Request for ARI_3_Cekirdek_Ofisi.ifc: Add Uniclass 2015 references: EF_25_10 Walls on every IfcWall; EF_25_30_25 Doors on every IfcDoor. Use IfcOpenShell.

First a look at what the model holds.

```python
import ifcopenshell

model = ifcopenshell.open("ARI_3_Cekirdek_Ofisi.ifc")
print(model.schema)
print("classifications:", [c.Name for c in model.by_type("IfcClassification")])
for ifc_class in ("IfcDoor", "IfcRoof", "IfcStair", "IfcWall", "IfcWindow"):
    print(ifc_class, len(model.by_type(ifc_class)))
```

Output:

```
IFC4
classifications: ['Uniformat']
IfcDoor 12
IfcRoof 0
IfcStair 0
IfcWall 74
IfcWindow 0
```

```python
import ifcopenshell
import ifcopenshell.api.classification

model = ifcopenshell.open("ARI_3_Cekirdek_Ofisi.ifc")

system = ifcopenshell.api.classification.add_classification(model, classification="Uniclass 2015")

codes = {
    "IfcWall": ("EF_25_10", "Walls"),
    "IfcDoor": ("EF_25_30_25", "Doors"),
}
for ifc_class, (code, name) in codes.items():
    products = model.by_type(ifc_class)
    ifcopenshell.api.classification.add_reference(
        model, products=products, classification=system, identification=code, name=name
    )
    print(code, len(products))

model.write("ARI_3_Cekirdek_Ofisi-out.ifc")
```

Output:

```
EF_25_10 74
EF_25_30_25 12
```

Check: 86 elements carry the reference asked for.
